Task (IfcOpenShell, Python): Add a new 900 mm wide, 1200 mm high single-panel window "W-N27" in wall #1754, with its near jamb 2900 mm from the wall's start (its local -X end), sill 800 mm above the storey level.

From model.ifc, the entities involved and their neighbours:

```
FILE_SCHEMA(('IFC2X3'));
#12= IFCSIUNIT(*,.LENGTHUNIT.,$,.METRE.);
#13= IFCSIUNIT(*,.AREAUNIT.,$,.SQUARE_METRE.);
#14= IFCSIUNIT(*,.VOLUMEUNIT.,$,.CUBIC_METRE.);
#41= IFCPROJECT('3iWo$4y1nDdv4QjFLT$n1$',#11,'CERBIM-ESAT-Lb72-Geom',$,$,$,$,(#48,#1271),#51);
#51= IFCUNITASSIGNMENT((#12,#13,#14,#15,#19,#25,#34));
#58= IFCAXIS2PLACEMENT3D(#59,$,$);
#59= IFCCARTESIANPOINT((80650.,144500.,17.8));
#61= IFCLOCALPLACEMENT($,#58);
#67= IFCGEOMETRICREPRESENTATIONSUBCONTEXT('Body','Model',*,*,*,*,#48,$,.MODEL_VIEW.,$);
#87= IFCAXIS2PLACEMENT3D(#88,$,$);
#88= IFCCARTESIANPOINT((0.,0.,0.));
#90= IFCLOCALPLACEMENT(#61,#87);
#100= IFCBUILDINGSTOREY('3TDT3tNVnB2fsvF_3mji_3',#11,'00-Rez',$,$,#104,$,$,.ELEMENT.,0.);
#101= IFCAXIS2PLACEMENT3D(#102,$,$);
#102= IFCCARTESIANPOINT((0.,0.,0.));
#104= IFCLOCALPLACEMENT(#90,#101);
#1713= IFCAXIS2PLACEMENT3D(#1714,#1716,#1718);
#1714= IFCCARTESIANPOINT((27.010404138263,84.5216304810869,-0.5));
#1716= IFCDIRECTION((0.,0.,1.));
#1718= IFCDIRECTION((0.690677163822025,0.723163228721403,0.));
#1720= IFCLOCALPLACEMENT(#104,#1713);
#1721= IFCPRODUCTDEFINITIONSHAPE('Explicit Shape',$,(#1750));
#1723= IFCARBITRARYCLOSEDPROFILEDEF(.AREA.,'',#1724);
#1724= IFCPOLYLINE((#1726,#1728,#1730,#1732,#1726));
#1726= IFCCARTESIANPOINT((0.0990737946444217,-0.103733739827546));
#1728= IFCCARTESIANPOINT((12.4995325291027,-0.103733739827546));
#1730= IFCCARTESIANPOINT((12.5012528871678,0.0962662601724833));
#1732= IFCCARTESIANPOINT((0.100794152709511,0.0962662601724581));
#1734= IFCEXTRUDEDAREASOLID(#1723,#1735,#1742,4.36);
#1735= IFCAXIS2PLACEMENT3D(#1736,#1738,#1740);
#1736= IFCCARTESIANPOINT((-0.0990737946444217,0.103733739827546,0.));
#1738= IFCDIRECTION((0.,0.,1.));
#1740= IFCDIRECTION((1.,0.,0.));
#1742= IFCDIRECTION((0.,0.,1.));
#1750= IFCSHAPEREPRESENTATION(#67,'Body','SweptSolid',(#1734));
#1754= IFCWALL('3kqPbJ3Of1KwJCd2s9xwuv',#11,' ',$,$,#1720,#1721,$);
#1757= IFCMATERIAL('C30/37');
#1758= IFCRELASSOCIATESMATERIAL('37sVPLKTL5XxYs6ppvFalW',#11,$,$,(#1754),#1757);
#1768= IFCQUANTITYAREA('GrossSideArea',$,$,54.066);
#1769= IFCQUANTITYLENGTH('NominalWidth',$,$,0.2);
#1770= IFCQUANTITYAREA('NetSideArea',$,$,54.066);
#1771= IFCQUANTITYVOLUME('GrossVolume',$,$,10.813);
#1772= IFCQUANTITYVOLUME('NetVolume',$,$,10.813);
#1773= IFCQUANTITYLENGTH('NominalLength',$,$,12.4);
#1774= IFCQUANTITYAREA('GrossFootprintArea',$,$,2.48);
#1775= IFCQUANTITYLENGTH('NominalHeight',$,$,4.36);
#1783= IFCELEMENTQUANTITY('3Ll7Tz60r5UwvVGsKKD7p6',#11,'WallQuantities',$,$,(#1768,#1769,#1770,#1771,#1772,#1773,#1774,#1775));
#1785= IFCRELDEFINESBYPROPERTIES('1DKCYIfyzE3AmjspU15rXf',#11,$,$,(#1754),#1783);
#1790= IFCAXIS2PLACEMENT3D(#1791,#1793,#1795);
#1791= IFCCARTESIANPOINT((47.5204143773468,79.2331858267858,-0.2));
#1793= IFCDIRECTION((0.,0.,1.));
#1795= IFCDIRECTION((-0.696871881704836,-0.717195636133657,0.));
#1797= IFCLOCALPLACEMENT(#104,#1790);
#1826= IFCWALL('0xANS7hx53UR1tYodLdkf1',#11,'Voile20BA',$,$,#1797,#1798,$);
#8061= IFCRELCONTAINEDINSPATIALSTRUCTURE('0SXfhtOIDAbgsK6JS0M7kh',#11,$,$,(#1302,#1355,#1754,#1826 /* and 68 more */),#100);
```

```python
import numpy as np
import ifcopenshell
import ifcopenshell.api.feature
import ifcopenshell.api.geometry
import ifcopenshell.api.pset
import ifcopenshell.api.root
import ifcopenshell.api.spatial
import ifcopenshell.api.type
import ifcopenshell.geom
import ifcopenshell.util.element
import ifcopenshell.util.placement
import ifcopenshell.util.representation
import ifcopenshell.util.shape
import ifcopenshell.util.unit

model = ifcopenshell.open("model.ifc")
unit_scale = ifcopenshell.util.unit.calculate_unit_scale(model)
area_scale = ifcopenshell.util.unit.calculate_unit_scale(model, "AREAUNIT")
volume_scale = ifcopenshell.util.unit.calculate_unit_scale(model, "VOLUMEUNIT")
settings = ifcopenshell.geom.settings()


def volume(element):
    """Net volume in cubic metres, openings subtracted."""
    shape = ifcopenshell.geom.create_shape(settings, element)
    return ifcopenshell.util.shape.get_volume(shape.geometry)


wall = model.by_id(1754)
storey = ifcopenshell.util.element.get_container(wall, ifc_class="IfcBuildingStorey")
context = ifcopenshell.util.representation.get_context(model, "Model", "Body", "MODEL_VIEW")
before = volume(wall)

width, height, from_end, sill = 0.9, 1.2, 2.9, 0.8  # metres

# The wall runs along its own X axis, and the end named is its -X end.
wall_shape = ifcopenshell.geom.create_shape(settings, wall)
x, y, z = ifcopenshell.util.shape.get_vertices(wall_shape.geometry).T
start = x.min() + from_end
face, thickness = float(y.min()), float(y.max() - y.min())
wall_matrix = ifcopenshell.util.placement.get_local_placement(wall.ObjectPlacement)
level = ifcopenshell.util.placement.get_local_placement(storey.ObjectPlacement)[2, 3]


def in_wall(x, y):
    """Placement at x, y metres in the wall's axes, at sill height."""
    matrix = wall_matrix.copy()
    matrix[:, 3] = wall_matrix @ np.array([x / unit_scale, y / unit_scale, 0.0, 1.0])
    matrix[2, 3] = level + sill / unit_scale
    return matrix


# Opening: a box that overshoots both wall faces by 50 mm.
opening = ifcopenshell.api.root.create_entity(model, ifc_class="IfcOpeningElement")
box = ifcopenshell.api.geometry.add_wall_representation(
    model, context=context, length=width, height=height, thickness=thickness + 0.1
)
ifcopenshell.api.geometry.assign_representation(model, product=opening, representation=box)
ifcopenshell.api.geometry.edit_object_placement(model, product=opening, matrix=in_wall(start, face - 0.05), is_si=False)
ifcopenshell.api.feature.add_feature(model, feature=opening, element=wall)

window = ifcopenshell.api.root.create_entity(model, ifc_class="IfcWindow", name="W-N27")
window.OverallWidth, window.OverallHeight = width / unit_scale, height / unit_scale
body = ifcopenshell.api.geometry.add_window_representation(
    model,
    context=context,
    overall_width=window.OverallWidth,
    overall_height=window.OverallHeight,
    partition_type="SINGLE_PANEL",
)
ifcopenshell.api.geometry.assign_representation(model, product=window, representation=body)
ifcopenshell.api.spatial.assign_container(model, products=[window], relating_structure=storey)
fills = ifcopenshell.api.feature.add_filling(model, opening=opening, element=window)
fills.OwnerHistory = window.OwnerHistory  # required in IFC2X3

# IFC2X3 keeps the operation on the window style.
style = ifcopenshell.api.root.create_entity(model, ifc_class="IfcWindowStyle", name="W-N27")
style.OperationType, style.ConstructionType = "SINGLE_PANEL", "NOTDEFINED"
style.ParameterTakesPrecedence = style.Sizeable = False
ifcopenshell.api.type.assign_type(model, related_objects=[window], relating_type=style)

# Centre the window in the wall's thickness.
ifcopenshell.api.geometry.edit_object_placement(model, product=window, matrix=in_wall(start, face), is_si=False)
window_shape = ifcopenshell.geom.create_shape(settings, window)
depth = ifcopenshell.util.shape.get_vertices(window_shape.geometry)[:, 1]
offset = face + thickness / 2 - (depth.min() + depth.max()) / 2
ifcopenshell.api.geometry.edit_object_placement(model, product=window, matrix=in_wall(start, offset), is_si=False)

after = volume(wall)

# Update the wall's stored quantities.
qto = model.by_id(ifcopenshell.util.element.get_pset(wall, "WallQuantities", should_inherit=False)["id"])
ifcopenshell.api.pset.edit_qto(model, qto=qto, properties={
    "NetSideArea": after / thickness / area_scale,
    "NetVolume": after / volume_scale,
})

print(f"wall volume {before:.3f} -> {after:.3f} m3")

model.write("model_v2.ifc")
```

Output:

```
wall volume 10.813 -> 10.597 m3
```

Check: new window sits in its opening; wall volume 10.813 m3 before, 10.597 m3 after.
